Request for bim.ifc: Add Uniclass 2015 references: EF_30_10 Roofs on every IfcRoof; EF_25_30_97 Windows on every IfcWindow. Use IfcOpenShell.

First a look at what the model holds.

```python
import ifcopenshell

model = ifcopenshell.open("bim.ifc")
print(model.schema)
print("classifications:", [c.Name for c in model.by_type("IfcClassification")])
for ifc_class in ("IfcDoor", "IfcRoof", "IfcStair", "IfcWall", "IfcWindow"):
    print(ifc_class, len(model.by_type(ifc_class)))
```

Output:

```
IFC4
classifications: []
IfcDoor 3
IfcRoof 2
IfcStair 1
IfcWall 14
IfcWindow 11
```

```python
import ifcopenshell
import ifcopenshell.api.classification

model = ifcopenshell.open("bim.ifc")

system = ifcopenshell.api.classification.add_classification(model, classification="Uniclass 2015")

codes = {
    "IfcRoof": ("EF_30_10", "Roofs"),
    "IfcWindow": ("EF_25_30_97", "Windows"),
}
for ifc_class, (code, name) in codes.items():
    products = model.by_type(ifc_class)
    ifcopenshell.api.classification.add_reference(
        model, products=products, classification=system, identification=code, name=name
    )
    print(code, len(products))

model.write("bim_rev.ifc")
```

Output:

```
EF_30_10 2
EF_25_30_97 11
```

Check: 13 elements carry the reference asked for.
